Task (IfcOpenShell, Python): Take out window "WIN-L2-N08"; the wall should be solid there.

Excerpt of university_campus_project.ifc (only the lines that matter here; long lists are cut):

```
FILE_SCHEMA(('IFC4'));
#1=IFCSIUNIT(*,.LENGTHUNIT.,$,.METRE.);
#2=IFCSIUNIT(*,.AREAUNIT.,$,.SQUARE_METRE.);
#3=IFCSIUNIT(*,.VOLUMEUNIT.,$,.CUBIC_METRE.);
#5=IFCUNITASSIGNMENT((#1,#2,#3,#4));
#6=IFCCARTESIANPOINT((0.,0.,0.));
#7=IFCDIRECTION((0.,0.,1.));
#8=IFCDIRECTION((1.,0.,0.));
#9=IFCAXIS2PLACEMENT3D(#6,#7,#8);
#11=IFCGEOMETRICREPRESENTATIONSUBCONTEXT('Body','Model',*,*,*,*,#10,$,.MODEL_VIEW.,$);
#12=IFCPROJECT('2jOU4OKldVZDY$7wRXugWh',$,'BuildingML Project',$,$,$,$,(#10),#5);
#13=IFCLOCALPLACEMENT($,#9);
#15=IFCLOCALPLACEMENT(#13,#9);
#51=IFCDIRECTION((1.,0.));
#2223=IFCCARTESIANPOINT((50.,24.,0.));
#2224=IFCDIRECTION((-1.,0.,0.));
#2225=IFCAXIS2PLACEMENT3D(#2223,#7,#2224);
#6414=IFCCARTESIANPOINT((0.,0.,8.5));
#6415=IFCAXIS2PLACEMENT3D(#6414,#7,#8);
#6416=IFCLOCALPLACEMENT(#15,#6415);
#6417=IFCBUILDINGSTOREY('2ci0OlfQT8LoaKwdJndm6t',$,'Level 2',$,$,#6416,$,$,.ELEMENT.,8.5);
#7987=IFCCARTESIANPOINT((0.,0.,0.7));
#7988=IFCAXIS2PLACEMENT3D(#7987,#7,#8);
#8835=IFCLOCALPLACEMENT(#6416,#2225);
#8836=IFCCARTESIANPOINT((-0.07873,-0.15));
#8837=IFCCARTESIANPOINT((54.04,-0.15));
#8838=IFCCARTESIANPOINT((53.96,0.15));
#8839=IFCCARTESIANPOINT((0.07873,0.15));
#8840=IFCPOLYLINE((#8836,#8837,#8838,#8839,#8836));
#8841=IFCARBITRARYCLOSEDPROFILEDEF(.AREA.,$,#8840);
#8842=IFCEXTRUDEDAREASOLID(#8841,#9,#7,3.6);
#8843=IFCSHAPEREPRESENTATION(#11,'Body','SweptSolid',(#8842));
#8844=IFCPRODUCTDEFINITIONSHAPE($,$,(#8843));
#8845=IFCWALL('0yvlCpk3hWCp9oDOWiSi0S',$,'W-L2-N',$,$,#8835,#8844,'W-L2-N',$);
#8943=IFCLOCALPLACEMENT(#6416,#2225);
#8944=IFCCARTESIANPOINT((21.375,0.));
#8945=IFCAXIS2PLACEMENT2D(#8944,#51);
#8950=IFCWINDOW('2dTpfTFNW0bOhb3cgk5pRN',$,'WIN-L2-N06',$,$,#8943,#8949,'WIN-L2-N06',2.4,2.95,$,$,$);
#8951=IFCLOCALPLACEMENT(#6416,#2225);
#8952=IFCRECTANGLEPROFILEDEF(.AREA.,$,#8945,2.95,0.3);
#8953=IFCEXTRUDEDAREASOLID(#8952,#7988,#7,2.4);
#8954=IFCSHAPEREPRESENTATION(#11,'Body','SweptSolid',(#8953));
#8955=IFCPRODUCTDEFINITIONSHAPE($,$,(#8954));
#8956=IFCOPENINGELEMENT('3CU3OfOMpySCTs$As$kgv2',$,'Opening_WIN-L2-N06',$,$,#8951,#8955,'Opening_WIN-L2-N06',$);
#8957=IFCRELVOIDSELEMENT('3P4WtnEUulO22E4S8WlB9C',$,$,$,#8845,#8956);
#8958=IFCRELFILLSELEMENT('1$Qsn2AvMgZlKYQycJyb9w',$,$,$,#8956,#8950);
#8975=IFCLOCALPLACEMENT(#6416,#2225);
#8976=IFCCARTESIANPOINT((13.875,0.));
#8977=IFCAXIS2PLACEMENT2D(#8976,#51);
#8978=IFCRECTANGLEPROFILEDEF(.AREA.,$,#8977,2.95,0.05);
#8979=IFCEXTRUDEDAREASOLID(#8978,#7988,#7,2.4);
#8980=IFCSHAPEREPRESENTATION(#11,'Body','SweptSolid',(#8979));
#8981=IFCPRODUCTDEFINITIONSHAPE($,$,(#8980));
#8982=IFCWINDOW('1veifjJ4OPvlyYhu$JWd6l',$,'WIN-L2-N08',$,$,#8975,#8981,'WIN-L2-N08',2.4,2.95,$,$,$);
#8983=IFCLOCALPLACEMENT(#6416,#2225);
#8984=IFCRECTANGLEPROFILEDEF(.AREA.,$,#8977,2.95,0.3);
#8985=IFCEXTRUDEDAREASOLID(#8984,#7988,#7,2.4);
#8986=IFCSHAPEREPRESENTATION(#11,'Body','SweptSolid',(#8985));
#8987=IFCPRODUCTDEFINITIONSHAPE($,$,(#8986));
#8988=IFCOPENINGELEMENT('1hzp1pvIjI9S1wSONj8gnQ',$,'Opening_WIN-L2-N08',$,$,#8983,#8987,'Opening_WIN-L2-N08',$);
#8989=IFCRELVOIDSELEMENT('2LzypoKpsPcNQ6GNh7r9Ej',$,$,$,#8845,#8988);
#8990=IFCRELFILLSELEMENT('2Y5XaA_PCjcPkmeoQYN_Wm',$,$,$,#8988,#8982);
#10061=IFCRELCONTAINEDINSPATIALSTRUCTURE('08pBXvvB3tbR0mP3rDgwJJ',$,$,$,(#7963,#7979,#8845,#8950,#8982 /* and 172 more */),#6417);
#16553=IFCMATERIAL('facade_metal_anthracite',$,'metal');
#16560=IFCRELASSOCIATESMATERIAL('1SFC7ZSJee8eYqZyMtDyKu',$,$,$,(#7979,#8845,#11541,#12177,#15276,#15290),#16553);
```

```python
import ifcopenshell
import ifcopenshell.api.feature
import ifcopenshell.api.root
import ifcopenshell.geom
import ifcopenshell.util.shape

model = ifcopenshell.open("university_campus_project.ifc")
settings = ifcopenshell.geom.settings()


def volume(element):
    """Net volume in cubic metres, openings subtracted."""
    shape = ifcopenshell.geom.create_shape(settings, element)
    return ifcopenshell.util.shape.get_volume(shape.geometry)


window = model.by_guid("1veifjJ4OPvlyYhu$JWd6l")
opening = window.FillsVoids[0].RelatingOpeningElement
wall = opening.VoidsElements[0].RelatingBuildingElement
before = volume(wall)

ifcopenshell.api.root.remove_product(model, product=window)
ifcopenshell.api.feature.remove_feature(model, feature=opening)

after = volume(wall)

print(f"wall volume {before:.3f} -> {after:.3f} m3")

model.write("university_campus_project_updated.ifc")
```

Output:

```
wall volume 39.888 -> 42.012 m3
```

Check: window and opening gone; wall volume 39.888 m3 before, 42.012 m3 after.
